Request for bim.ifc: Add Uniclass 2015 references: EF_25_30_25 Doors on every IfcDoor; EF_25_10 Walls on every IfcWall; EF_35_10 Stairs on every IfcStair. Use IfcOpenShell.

First a look at what the model holds.

```python
import ifcopenshell

model = ifcopenshell.open("bim.ifc")
print(model.schema)
print("classifications:", [c.Name for c in model.by_type("IfcClassification")])
for ifc_class in ("IfcDoor", "IfcRoof", "IfcStair", "IfcWall", "IfcWindow"):
    print(ifc_class, len(model.by_type(ifc_class)))
```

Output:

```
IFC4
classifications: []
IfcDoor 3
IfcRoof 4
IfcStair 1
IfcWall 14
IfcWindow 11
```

```python
import ifcopenshell
import ifcopenshell.api.classification

model = ifcopenshell.open("bim.ifc")

system = ifcopenshell.api.classification.add_classification(model, classification="Uniclass 2015")

codes = {
    "IfcDoor": ("EF_25_30_25", "Doors"),
    "IfcWall": ("EF_25_10", "Walls"),
    "IfcStair": ("EF_35_10", "Stairs"),
}
for ifc_class, (code, name) in codes.items():
    products = model.by_type(ifc_class)
    ifcopenshell.api.classification.add_reference(
        model, products=products, classification=system, identification=code, name=name
    )
    print(code, len(products))

model.write("bim_rev.ifc")
```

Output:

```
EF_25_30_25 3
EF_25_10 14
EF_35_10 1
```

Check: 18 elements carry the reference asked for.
